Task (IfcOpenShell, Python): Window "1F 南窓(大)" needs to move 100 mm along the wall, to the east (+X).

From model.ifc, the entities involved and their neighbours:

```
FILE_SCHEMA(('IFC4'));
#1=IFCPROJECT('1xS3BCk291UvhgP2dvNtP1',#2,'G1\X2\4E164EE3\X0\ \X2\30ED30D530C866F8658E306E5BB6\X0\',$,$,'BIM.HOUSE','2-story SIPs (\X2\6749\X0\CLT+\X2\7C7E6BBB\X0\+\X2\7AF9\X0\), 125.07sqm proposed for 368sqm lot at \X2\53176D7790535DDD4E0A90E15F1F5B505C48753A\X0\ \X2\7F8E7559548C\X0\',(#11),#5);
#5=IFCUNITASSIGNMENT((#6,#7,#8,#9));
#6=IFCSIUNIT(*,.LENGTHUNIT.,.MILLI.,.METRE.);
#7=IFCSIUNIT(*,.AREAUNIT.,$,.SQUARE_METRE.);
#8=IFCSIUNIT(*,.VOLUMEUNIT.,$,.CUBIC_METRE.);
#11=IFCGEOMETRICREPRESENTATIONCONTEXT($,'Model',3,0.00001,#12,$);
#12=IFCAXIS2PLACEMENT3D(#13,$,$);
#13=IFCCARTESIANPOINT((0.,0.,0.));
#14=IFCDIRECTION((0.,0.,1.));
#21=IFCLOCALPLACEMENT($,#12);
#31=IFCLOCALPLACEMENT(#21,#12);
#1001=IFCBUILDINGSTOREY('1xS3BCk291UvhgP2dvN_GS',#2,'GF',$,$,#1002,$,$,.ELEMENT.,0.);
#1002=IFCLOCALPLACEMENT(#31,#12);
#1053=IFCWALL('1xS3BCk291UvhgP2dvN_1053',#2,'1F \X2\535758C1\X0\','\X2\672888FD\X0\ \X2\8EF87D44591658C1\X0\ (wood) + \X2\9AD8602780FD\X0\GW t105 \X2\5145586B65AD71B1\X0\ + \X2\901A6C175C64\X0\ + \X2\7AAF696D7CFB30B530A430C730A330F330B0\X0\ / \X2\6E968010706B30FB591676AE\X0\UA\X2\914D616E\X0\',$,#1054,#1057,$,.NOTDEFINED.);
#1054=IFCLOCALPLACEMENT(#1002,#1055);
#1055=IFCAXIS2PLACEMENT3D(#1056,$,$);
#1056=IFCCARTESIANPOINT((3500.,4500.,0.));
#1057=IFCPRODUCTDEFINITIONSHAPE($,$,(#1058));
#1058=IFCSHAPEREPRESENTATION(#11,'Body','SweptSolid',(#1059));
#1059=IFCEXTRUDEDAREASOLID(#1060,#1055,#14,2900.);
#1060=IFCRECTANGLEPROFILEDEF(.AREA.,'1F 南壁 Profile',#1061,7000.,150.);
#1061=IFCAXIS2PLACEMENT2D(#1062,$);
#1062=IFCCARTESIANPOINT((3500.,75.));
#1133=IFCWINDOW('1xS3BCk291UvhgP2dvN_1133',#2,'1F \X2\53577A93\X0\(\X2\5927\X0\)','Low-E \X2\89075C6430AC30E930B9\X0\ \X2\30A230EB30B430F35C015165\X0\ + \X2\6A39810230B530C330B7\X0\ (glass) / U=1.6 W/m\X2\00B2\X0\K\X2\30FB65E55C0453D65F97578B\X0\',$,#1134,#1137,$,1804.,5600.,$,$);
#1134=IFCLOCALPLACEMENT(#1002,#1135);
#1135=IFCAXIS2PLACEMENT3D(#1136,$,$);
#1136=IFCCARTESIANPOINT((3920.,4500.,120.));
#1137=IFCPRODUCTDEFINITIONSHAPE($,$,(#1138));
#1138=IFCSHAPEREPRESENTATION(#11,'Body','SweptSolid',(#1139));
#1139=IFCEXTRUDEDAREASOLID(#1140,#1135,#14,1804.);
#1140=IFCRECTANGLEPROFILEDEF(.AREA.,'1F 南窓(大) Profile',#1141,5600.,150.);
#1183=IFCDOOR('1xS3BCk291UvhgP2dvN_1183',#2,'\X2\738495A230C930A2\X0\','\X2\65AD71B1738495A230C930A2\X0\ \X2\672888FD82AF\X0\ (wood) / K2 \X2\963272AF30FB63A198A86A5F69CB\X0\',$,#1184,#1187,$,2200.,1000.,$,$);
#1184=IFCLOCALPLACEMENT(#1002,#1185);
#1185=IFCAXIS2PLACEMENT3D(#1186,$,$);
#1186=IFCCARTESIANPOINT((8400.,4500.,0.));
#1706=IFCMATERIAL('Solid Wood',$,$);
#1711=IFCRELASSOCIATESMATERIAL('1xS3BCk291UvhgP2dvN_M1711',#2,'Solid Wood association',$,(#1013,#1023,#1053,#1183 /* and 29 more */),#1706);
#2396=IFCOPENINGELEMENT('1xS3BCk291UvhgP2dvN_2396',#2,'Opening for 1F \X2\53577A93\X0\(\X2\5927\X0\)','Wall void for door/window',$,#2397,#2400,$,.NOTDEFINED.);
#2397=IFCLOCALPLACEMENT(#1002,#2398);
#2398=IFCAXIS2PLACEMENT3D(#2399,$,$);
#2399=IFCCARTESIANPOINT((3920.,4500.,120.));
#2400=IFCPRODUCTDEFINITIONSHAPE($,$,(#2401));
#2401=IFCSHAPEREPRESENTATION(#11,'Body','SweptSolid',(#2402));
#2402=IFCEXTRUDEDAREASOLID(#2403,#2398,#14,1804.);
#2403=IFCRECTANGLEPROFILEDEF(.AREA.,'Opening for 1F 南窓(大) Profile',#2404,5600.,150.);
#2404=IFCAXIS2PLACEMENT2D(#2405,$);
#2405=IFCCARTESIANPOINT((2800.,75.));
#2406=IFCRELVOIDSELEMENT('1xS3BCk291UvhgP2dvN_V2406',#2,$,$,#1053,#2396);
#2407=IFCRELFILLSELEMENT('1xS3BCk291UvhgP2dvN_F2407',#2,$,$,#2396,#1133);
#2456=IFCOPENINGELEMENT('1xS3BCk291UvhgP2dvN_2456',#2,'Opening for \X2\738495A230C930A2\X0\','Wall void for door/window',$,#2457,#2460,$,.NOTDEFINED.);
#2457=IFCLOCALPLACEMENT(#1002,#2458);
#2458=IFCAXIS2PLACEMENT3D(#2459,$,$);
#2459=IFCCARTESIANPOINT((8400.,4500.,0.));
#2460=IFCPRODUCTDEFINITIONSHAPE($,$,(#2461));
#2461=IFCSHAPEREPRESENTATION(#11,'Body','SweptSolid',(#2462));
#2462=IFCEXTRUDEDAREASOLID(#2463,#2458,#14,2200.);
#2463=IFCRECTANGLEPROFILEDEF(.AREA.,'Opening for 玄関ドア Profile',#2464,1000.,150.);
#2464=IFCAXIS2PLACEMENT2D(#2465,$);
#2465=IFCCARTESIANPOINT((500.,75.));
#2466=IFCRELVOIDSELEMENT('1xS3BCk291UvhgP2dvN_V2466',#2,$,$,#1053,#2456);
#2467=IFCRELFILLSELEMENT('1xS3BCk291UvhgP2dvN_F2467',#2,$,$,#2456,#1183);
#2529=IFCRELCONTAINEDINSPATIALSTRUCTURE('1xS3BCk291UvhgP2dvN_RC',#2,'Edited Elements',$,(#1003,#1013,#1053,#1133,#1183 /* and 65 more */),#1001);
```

```python
import ifcopenshell
import ifcopenshell.api.geometry
import ifcopenshell.util.placement

model = ifcopenshell.open("model.ifc")

window = model.by_id(1133)
opening = window.FillsVoids[0].RelatingOpeningElement
wall = opening.VoidsElements[0].RelatingBuildingElement

wall_matrix = ifcopenshell.util.placement.get_local_placement(wall.ObjectPlacement)
shift = wall_matrix[:3, 0] * 100.0
before = ifcopenshell.util.placement.get_local_placement(window.ObjectPlacement)[:3, 3].copy()

# The window is not placed relative to its opening, so move both.
for product in (opening, window):
    matrix = ifcopenshell.util.placement.get_local_placement(product.ObjectPlacement)
    matrix[:3, 3] += shift
    ifcopenshell.api.geometry.edit_object_placement(model, product=product, matrix=matrix, is_si=False)

after = ifcopenshell.util.placement.get_local_placement(window.ObjectPlacement)[:3, 3]
print("window moved by", (after - before).round(3) + 0.0)

model.write("model_v2.ifc")
```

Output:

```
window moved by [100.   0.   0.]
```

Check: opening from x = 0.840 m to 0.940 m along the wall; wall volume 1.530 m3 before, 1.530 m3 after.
